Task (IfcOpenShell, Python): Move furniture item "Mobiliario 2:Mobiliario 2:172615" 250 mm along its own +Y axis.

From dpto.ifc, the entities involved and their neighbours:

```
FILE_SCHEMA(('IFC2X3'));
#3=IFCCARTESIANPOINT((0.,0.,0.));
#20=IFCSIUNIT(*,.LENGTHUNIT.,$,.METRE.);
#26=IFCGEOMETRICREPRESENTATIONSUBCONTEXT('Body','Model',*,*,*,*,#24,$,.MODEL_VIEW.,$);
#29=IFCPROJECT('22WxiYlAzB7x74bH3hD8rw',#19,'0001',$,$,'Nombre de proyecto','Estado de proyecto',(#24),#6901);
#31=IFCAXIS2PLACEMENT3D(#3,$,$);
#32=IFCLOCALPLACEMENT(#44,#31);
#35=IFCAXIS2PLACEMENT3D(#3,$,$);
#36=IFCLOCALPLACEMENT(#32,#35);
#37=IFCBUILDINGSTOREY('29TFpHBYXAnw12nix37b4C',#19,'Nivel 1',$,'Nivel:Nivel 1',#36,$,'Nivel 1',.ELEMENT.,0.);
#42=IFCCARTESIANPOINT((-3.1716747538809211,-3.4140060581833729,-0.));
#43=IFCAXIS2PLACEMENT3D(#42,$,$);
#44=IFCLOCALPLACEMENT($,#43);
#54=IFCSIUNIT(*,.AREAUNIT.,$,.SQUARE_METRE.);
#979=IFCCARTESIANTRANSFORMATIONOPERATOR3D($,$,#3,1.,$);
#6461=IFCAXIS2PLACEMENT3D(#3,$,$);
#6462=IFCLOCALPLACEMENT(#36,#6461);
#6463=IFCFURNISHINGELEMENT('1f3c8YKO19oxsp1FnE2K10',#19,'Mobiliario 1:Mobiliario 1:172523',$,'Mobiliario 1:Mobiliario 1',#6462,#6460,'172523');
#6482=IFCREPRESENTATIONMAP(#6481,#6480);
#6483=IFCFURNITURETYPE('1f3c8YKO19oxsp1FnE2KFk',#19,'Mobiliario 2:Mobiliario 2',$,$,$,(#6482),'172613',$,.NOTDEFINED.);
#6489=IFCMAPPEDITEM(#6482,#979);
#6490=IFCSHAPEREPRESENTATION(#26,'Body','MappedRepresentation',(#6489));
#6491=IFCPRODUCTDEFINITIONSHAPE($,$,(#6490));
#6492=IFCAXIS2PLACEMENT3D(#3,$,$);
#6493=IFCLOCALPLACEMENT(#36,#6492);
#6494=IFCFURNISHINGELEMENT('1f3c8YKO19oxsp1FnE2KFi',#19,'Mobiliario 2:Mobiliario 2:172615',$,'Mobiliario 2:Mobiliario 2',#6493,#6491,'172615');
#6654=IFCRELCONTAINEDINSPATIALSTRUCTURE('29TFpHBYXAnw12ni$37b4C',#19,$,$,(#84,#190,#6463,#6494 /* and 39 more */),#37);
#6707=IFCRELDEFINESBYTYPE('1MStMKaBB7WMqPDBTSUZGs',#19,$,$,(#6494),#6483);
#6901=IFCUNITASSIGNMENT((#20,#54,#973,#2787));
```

```python
import ifcopenshell
import ifcopenshell.api.geometry
import ifcopenshell.util.placement
import ifcopenshell.util.unit

model = ifcopenshell.open("dpto.ifc")
unit_scale = ifcopenshell.util.unit.calculate_unit_scale(model)

item = model.by_id(6494)
matrix = ifcopenshell.util.placement.get_local_placement(item.ObjectPlacement)
matrix[:3, 3] += matrix[:3, 1] * 0.25 / unit_scale
ifcopenshell.api.geometry.edit_object_placement(model, product=item, matrix=matrix, is_si=False)

print(ifcopenshell.util.placement.get_local_placement(item.ObjectPlacement).round(3) + 0.0)

model.write("dpto_edited.ifc")
```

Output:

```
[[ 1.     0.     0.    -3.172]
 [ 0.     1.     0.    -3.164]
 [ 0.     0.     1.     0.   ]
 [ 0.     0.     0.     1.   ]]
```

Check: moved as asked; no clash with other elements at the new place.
